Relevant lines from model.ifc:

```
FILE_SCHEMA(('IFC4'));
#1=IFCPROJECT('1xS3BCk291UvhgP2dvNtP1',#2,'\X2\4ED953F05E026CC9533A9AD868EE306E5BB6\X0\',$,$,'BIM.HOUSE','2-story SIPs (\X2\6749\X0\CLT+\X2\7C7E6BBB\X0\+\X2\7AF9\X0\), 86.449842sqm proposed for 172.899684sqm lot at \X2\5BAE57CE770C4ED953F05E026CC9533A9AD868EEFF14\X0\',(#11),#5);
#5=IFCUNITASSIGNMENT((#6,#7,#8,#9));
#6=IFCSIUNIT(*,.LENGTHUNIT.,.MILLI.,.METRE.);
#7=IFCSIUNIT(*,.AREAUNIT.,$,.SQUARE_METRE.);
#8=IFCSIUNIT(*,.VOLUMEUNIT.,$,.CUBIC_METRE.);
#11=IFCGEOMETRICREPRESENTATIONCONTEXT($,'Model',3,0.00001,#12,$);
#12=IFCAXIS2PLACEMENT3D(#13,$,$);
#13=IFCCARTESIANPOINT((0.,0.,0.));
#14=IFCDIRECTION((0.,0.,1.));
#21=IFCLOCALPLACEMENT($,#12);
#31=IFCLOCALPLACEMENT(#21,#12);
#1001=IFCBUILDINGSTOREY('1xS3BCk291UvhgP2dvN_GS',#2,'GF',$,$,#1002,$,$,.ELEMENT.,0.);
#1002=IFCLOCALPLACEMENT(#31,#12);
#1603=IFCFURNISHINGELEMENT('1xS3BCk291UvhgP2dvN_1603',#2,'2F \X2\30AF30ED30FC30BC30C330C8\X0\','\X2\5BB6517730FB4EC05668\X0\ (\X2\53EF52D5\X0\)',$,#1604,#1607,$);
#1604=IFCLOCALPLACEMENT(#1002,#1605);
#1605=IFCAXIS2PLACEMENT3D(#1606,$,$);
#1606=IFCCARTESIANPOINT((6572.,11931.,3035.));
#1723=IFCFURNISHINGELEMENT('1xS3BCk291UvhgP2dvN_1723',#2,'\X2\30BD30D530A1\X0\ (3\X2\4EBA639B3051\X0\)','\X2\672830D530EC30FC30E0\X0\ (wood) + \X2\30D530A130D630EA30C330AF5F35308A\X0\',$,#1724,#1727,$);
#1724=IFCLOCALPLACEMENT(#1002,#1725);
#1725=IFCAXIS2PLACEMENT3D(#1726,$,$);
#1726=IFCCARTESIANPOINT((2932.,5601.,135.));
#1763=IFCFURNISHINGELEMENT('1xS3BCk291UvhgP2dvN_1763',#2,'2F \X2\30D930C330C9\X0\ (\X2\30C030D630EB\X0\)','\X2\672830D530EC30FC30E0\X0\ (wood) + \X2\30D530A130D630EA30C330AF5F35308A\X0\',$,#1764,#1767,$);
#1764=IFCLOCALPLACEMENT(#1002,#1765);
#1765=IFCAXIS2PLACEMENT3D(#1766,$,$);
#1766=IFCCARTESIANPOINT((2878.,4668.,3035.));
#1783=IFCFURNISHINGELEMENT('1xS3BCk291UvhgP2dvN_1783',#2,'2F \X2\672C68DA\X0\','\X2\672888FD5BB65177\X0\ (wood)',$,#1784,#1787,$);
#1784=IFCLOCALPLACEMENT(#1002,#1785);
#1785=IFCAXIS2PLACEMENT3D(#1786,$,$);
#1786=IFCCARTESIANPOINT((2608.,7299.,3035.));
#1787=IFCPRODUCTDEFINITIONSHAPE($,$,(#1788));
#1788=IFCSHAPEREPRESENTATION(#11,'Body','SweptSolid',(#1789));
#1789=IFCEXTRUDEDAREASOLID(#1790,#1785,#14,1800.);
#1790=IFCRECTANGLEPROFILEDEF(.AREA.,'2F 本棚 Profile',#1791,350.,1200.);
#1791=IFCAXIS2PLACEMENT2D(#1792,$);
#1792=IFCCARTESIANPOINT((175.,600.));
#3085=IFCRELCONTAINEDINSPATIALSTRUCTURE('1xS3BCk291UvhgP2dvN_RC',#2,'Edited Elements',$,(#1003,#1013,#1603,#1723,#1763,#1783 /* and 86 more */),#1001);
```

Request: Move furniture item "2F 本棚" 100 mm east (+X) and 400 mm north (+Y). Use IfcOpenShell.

```python
import ifcopenshell
import ifcopenshell.api.geometry
import ifcopenshell.util.placement

model = ifcopenshell.open("model.ifc")

item = model.by_guid("1xS3BCk291UvhgP2dvN_1783")
matrix = ifcopenshell.util.placement.get_local_placement(item.ObjectPlacement)
matrix[0, 3] += 100.0
matrix[1, 3] += 400.0
ifcopenshell.api.geometry.edit_object_placement(model, product=item, matrix=matrix, is_si=False)

print(ifcopenshell.util.placement.get_local_placement(item.ObjectPlacement).round(3) + 0.0)

model.write("model-out.ifc")
```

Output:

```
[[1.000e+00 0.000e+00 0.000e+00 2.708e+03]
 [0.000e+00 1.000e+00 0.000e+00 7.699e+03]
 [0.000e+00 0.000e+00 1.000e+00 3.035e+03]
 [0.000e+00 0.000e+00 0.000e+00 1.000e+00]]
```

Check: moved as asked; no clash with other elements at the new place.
